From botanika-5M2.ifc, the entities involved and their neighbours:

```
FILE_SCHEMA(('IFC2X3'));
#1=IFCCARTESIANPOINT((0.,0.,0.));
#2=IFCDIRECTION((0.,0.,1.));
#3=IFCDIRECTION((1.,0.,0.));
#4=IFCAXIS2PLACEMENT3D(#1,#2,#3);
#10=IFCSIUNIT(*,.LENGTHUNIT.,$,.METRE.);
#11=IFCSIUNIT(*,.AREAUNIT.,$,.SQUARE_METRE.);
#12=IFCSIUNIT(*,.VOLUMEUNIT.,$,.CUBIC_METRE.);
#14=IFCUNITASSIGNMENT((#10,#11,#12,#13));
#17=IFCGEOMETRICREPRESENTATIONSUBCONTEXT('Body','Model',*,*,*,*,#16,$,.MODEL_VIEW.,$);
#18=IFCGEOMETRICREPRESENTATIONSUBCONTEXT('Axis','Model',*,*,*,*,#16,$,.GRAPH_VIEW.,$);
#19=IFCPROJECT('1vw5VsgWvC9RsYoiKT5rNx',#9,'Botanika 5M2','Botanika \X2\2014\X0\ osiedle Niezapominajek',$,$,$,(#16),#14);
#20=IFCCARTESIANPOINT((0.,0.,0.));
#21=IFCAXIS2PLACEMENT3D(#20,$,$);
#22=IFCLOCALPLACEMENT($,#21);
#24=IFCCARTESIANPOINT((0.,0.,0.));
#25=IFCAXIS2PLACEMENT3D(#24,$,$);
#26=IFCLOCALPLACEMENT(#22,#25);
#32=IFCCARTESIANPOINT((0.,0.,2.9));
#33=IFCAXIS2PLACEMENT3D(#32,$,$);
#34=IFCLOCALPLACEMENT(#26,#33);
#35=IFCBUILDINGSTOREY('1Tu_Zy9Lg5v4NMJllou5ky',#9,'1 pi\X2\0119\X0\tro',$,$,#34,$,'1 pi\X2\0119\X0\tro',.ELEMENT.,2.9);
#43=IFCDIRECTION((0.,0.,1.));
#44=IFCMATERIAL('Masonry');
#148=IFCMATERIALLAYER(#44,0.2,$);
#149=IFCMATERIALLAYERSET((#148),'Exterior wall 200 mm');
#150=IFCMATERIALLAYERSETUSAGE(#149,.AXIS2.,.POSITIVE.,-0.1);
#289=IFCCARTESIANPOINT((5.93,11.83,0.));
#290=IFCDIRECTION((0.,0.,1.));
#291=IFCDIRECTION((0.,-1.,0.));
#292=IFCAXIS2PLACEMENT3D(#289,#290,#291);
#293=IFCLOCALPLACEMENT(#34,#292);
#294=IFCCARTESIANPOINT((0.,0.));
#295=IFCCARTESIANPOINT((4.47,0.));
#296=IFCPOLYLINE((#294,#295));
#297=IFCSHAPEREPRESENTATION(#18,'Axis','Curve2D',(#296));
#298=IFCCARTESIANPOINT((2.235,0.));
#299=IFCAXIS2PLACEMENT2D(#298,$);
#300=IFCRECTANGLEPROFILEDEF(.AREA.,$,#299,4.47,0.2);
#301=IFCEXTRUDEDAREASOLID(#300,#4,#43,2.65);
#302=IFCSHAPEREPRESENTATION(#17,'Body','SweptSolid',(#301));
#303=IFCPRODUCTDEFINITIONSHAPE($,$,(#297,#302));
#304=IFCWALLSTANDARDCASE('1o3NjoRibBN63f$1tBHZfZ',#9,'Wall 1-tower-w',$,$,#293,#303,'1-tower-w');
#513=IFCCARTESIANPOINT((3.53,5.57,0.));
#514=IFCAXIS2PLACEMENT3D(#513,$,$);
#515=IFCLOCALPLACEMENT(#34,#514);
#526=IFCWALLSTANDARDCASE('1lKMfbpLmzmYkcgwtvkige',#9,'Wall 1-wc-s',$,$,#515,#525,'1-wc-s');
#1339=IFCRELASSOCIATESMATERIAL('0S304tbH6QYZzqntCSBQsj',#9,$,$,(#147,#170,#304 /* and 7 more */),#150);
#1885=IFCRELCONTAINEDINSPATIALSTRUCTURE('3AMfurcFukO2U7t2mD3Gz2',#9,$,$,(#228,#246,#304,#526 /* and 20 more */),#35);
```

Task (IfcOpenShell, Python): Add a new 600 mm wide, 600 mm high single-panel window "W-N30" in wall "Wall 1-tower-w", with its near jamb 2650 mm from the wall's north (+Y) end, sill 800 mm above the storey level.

```python
import numpy as np
import ifcopenshell
import ifcopenshell.api.feature
import ifcopenshell.api.geometry
import ifcopenshell.api.root
import ifcopenshell.api.spatial
import ifcopenshell.api.type
import ifcopenshell.geom
import ifcopenshell.util.element
import ifcopenshell.util.placement
import ifcopenshell.util.representation
import ifcopenshell.util.shape
import ifcopenshell.util.unit

model = ifcopenshell.open("botanika-5M2.ifc")
unit_scale = ifcopenshell.util.unit.calculate_unit_scale(model)
settings = ifcopenshell.geom.settings()


def volume(element):
    """Net volume in cubic metres, openings subtracted."""
    shape = ifcopenshell.geom.create_shape(settings, element)
    return ifcopenshell.util.shape.get_volume(shape.geometry)


wall = model.by_guid("1o3NjoRibBN63f$1tBHZfZ")
storey = ifcopenshell.util.element.get_container(wall, ifc_class="IfcBuildingStorey")
context = ifcopenshell.util.representation.get_context(model, "Model", "Body", "MODEL_VIEW")
before = volume(wall)

width, height, from_end, sill = 0.6, 0.6, 2.65, 0.8  # metres

# The wall runs along its own X axis, and the end named is its -X end.
wall_shape = ifcopenshell.geom.create_shape(settings, wall)
x, y, z = ifcopenshell.util.shape.get_vertices(wall_shape.geometry).T
start = x.min() + from_end
face, thickness = float(y.min()), float(y.max() - y.min())
wall_matrix = ifcopenshell.util.placement.get_local_placement(wall.ObjectPlacement)
level = ifcopenshell.util.placement.get_local_placement(storey.ObjectPlacement)[2, 3]


def in_wall(x, y):
    """Placement at x, y metres in the wall's axes, at sill height."""
    matrix = wall_matrix.copy()
    matrix[:, 3] = wall_matrix @ np.array([x / unit_scale, y / unit_scale, 0.0, 1.0])
    matrix[2, 3] = level + sill / unit_scale
    return matrix


# Opening: a box that overshoots both wall faces by 50 mm.
opening = ifcopenshell.api.root.create_entity(model, ifc_class="IfcOpeningElement")
box = ifcopenshell.api.geometry.add_wall_representation(
    model, context=context, length=width, height=height, thickness=thickness + 0.1
)
ifcopenshell.api.geometry.assign_representation(model, product=opening, representation=box)
ifcopenshell.api.geometry.edit_object_placement(model, product=opening, matrix=in_wall(start, face - 0.05), is_si=False)
ifcopenshell.api.feature.add_feature(model, feature=opening, element=wall)

window = ifcopenshell.api.root.create_entity(model, ifc_class="IfcWindow", name="W-N30")
window.OverallWidth, window.OverallHeight = width / unit_scale, height / unit_scale
body = ifcopenshell.api.geometry.add_window_representation(
    model,
    context=context,
    overall_width=window.OverallWidth,
    overall_height=window.OverallHeight,
    partition_type="SINGLE_PANEL",
)
ifcopenshell.api.geometry.assign_representation(model, product=window, representation=body)
ifcopenshell.api.spatial.assign_container(model, products=[window], relating_structure=storey)
fills = ifcopenshell.api.feature.add_filling(model, opening=opening, element=window)
fills.OwnerHistory = window.OwnerHistory  # required in IFC2X3

# IFC2X3 keeps the operation on the window style.
style = ifcopenshell.api.root.create_entity(model, ifc_class="IfcWindowStyle", name="W-N30")
style.OperationType, style.ConstructionType = "SINGLE_PANEL", "NOTDEFINED"
style.ParameterTakesPrecedence = style.Sizeable = False
ifcopenshell.api.type.assign_type(model, related_objects=[window], relating_type=style)

# Centre the window in the wall's thickness.
ifcopenshell.api.geometry.edit_object_placement(model, product=window, matrix=in_wall(start, face), is_si=False)
window_shape = ifcopenshell.geom.create_shape(settings, window)
depth = ifcopenshell.util.shape.get_vertices(window_shape.geometry)[:, 1]
offset = face + thickness / 2 - (depth.min() + depth.max()) / 2
ifcopenshell.api.geometry.edit_object_placement(model, product=window, matrix=in_wall(start, offset), is_si=False)

after = volume(wall)

print(f"wall volume {before:.3f} -> {after:.3f} m3")

model.write("botanika-5M2_edited.ifc")
```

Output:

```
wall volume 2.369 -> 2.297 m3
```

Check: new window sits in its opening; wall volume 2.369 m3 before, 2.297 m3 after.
